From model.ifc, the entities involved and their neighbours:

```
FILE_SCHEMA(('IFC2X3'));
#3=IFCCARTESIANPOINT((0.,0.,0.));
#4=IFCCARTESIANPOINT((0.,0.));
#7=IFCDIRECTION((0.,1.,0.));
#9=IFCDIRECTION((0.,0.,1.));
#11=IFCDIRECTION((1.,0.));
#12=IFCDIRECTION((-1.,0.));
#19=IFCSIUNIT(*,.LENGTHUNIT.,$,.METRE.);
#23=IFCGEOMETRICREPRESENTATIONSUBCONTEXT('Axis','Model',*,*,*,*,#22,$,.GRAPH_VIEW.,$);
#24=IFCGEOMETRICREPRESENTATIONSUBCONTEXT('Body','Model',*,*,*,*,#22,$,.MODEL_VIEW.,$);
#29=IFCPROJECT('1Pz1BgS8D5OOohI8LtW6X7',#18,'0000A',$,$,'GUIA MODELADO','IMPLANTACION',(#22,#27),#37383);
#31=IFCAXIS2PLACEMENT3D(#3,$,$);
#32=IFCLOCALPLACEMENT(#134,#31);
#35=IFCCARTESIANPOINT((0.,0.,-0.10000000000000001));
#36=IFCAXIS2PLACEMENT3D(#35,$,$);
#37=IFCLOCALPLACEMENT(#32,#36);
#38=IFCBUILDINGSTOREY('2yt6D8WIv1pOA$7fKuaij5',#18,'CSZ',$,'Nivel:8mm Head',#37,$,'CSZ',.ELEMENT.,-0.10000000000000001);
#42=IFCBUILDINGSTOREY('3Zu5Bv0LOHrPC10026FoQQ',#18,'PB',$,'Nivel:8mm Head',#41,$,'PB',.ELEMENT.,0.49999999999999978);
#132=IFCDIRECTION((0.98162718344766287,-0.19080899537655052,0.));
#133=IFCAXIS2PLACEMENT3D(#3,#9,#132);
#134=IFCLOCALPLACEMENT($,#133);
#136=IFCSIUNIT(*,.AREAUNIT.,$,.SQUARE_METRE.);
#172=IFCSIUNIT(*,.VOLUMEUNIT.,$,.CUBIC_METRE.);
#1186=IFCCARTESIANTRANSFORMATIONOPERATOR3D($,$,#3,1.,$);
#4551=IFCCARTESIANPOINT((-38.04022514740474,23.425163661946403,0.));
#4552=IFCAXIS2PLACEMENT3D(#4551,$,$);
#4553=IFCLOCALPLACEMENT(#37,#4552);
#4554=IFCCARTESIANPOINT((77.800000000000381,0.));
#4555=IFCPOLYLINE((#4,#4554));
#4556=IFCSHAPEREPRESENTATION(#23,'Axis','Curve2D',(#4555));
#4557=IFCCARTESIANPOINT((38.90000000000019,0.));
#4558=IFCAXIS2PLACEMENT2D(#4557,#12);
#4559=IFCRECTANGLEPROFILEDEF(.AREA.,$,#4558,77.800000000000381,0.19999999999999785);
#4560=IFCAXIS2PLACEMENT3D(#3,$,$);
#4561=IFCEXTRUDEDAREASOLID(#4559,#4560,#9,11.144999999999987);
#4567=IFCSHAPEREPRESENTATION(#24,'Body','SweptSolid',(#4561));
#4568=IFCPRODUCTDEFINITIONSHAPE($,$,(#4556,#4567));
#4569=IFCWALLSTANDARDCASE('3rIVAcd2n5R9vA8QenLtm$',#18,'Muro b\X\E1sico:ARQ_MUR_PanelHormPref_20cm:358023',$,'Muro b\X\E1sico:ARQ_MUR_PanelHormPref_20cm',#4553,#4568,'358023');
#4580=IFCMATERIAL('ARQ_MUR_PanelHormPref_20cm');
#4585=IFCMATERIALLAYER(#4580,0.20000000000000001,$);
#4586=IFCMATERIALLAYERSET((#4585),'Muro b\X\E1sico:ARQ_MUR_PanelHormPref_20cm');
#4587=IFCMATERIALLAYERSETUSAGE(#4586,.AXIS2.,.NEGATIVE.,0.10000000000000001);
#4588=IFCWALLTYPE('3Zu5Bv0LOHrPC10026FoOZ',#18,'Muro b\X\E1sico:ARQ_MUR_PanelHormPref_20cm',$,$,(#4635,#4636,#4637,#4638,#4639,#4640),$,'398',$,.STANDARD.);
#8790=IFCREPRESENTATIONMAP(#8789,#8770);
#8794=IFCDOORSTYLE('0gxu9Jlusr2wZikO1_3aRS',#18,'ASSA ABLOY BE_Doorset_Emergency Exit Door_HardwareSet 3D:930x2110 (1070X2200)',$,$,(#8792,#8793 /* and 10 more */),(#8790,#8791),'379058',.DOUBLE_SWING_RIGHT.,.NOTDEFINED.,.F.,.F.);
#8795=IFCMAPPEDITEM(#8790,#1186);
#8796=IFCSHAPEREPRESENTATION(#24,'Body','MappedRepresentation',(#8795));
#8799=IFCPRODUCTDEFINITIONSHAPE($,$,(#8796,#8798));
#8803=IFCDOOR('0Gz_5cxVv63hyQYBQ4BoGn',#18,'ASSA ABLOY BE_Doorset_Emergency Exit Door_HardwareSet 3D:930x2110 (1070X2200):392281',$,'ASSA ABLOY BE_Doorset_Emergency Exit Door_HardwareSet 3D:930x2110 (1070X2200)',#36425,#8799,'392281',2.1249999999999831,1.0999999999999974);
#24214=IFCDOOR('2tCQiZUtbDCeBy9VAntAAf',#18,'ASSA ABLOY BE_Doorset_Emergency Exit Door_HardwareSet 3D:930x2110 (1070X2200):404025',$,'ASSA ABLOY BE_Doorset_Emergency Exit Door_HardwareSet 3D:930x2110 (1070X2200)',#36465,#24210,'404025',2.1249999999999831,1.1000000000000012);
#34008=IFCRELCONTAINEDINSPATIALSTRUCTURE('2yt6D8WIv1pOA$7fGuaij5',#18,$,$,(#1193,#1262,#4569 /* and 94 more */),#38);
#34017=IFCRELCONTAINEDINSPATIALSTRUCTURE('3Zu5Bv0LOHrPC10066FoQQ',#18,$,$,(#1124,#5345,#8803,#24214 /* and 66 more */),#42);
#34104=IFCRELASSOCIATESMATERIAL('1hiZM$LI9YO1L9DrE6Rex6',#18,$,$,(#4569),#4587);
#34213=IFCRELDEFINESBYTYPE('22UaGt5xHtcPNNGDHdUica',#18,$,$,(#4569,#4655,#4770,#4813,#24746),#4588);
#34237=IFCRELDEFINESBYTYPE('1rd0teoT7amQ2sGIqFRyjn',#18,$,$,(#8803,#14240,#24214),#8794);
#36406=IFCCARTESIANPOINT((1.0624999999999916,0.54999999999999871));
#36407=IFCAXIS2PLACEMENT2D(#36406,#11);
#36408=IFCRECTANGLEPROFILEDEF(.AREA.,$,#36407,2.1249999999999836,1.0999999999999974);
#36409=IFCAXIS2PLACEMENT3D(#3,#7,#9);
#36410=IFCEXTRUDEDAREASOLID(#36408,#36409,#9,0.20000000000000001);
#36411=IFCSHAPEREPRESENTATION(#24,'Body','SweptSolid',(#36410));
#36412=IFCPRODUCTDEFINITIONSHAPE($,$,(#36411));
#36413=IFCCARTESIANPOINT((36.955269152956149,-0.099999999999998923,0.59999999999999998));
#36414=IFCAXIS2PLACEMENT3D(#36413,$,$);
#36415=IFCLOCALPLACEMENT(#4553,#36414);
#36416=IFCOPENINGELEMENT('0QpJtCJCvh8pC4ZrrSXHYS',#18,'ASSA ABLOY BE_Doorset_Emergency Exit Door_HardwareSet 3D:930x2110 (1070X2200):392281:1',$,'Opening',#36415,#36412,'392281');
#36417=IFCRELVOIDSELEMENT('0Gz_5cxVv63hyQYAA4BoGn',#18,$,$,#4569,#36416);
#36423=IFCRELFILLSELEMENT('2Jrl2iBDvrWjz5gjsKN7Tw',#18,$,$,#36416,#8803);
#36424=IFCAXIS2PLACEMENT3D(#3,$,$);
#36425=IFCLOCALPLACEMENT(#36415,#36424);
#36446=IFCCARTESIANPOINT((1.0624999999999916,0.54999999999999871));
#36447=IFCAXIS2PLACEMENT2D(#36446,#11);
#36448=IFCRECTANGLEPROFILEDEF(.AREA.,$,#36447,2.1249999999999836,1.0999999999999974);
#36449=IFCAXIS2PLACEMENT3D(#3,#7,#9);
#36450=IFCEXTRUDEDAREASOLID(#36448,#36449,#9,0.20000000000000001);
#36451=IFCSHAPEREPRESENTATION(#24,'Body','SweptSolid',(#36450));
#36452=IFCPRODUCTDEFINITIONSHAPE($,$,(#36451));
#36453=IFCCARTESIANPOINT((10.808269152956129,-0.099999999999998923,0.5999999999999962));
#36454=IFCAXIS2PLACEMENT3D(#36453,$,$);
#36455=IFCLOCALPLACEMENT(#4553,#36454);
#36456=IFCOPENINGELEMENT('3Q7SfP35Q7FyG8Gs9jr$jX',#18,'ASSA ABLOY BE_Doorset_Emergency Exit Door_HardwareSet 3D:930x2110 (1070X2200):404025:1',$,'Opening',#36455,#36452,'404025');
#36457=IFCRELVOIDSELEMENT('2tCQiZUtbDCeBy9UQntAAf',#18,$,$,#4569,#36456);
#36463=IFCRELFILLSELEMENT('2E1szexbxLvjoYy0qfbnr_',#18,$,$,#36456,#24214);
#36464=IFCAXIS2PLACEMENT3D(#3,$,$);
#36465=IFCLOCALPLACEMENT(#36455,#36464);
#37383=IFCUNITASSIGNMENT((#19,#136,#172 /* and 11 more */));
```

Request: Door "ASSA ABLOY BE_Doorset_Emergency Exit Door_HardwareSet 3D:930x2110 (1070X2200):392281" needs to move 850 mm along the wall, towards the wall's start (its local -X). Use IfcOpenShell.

```python
import ifcopenshell
import ifcopenshell.api.geometry
import ifcopenshell.util.placement

model = ifcopenshell.open("model.ifc")

door = model.by_guid("0Gz_5cxVv63hyQYBQ4BoGn")
opening = door.FillsVoids[0].RelatingOpeningElement
wall = opening.VoidsElements[0].RelatingBuildingElement

wall_matrix = ifcopenshell.util.placement.get_local_placement(wall.ObjectPlacement)
shift = wall_matrix[:3, 0] * -0.85
before = ifcopenshell.util.placement.get_local_placement(door.ObjectPlacement)[:3, 3].copy()

# The door is placed relative to its opening, so it follows when the opening moves.
matrix = ifcopenshell.util.placement.get_local_placement(opening.ObjectPlacement)
matrix[:3, 3] += shift
ifcopenshell.api.geometry.edit_object_placement(
    model, product=opening, matrix=matrix, is_si=False, should_transform_children=True
)

after = ifcopenshell.util.placement.get_local_placement(door.ObjectPlacement)[:3, 3]
print("door moved by", (after - before).round(3) + 0.0)

model.write("model_edited.ifc")
```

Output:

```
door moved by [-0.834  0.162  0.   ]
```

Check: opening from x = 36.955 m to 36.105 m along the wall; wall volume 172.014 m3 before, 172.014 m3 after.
